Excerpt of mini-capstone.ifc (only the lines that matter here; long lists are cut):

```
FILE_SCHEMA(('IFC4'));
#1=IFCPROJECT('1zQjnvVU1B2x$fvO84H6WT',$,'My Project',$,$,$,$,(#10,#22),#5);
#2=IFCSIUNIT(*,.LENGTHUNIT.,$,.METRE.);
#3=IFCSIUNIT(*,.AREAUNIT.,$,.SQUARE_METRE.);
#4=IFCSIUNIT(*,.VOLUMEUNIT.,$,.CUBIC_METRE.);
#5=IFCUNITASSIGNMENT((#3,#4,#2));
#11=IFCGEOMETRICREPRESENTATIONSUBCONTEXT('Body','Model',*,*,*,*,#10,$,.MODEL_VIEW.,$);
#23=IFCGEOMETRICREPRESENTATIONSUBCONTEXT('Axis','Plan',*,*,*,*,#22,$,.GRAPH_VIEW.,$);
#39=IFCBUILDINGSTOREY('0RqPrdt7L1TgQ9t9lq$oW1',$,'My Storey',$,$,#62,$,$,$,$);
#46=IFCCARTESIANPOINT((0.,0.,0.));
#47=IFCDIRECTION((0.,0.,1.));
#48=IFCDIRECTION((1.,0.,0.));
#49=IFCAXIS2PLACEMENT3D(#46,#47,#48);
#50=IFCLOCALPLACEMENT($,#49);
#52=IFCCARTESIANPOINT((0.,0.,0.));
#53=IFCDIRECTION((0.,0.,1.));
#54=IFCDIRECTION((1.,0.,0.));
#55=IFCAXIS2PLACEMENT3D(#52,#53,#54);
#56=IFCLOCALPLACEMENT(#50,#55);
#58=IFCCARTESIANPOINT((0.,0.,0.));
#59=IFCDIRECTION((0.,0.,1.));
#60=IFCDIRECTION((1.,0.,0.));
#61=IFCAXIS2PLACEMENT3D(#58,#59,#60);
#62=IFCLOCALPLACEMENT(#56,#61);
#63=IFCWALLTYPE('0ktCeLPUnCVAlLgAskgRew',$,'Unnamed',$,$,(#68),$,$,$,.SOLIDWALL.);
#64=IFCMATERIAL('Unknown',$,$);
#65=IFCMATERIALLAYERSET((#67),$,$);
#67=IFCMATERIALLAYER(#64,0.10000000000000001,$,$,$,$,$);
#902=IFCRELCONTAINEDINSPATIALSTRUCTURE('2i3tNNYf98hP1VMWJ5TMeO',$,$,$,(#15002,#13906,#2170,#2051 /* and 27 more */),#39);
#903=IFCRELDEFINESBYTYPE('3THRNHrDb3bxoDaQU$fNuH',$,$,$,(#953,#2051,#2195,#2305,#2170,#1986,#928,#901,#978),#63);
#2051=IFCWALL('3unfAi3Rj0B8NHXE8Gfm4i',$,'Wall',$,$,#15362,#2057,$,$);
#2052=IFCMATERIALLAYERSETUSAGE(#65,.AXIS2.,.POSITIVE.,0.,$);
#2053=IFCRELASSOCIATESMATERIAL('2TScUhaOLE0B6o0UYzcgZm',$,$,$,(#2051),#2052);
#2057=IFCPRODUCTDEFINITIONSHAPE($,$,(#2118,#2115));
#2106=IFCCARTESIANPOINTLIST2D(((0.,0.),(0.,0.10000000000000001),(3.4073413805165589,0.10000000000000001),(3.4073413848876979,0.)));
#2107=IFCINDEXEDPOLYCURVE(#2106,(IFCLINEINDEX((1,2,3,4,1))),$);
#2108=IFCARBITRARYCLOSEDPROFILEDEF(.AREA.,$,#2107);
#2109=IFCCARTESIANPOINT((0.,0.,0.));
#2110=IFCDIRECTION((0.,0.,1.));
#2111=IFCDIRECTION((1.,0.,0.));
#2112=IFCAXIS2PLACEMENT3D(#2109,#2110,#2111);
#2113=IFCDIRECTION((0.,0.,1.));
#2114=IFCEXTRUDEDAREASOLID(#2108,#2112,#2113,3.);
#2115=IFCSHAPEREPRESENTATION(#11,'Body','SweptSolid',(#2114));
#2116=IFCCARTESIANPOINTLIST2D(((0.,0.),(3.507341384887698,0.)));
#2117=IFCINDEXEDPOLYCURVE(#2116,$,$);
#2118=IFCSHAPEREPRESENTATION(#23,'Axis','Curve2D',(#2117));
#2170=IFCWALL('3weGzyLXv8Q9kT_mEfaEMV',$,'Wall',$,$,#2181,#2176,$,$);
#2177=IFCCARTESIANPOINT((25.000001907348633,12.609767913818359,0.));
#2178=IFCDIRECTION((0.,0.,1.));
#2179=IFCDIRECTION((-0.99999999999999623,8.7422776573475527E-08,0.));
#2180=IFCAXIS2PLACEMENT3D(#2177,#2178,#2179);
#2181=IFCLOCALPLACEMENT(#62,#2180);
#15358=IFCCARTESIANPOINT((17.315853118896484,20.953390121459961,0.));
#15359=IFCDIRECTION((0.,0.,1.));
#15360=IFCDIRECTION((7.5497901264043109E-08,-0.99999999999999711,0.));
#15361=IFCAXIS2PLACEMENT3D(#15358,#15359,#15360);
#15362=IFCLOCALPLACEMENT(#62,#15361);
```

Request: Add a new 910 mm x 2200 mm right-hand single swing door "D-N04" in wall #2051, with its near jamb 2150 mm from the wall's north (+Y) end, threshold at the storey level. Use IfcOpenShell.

```python
import numpy as np
import ifcopenshell
import ifcopenshell.api.feature
import ifcopenshell.api.geometry
import ifcopenshell.api.root
import ifcopenshell.api.spatial
import ifcopenshell.geom
import ifcopenshell.util.element
import ifcopenshell.util.placement
import ifcopenshell.util.representation
import ifcopenshell.util.shape
import ifcopenshell.util.unit

model = ifcopenshell.open("mini-capstone.ifc")
unit_scale = ifcopenshell.util.unit.calculate_unit_scale(model)
settings = ifcopenshell.geom.settings()


def volume(element):
    """Net volume in cubic metres, openings subtracted."""
    shape = ifcopenshell.geom.create_shape(settings, element)
    return ifcopenshell.util.shape.get_volume(shape.geometry)


wall = model.by_id(2051)
storey = ifcopenshell.util.element.get_container(wall, ifc_class="IfcBuildingStorey")
context = ifcopenshell.util.representation.get_context(model, "Model", "Body", "MODEL_VIEW")
before = volume(wall)

width, height, from_end, sill = 0.91, 2.2, 2.15, 0.0  # metres

# The wall runs along its own X axis, and the end named is its -X end.
wall_shape = ifcopenshell.geom.create_shape(settings, wall)
x, y, z = ifcopenshell.util.shape.get_vertices(wall_shape.geometry).T
start = x.min() + from_end
face, thickness = float(y.min()), float(y.max() - y.min())
wall_matrix = ifcopenshell.util.placement.get_local_placement(wall.ObjectPlacement)
level = ifcopenshell.util.placement.get_local_placement(storey.ObjectPlacement)[2, 3]


def in_wall(x, y):
    """Placement at x, y metres in the wall's axes, at sill height."""
    matrix = wall_matrix.copy()
    matrix[:, 3] = wall_matrix @ np.array([x / unit_scale, y / unit_scale, 0.0, 1.0])
    matrix[2, 3] = level + sill / unit_scale
    return matrix


# Opening: a box that overshoots both wall faces by 50 mm.
opening = ifcopenshell.api.root.create_entity(model, ifc_class="IfcOpeningElement", predefined_type="OPENING")
box = ifcopenshell.api.geometry.add_wall_representation(
    model, context=context, length=width, height=height, thickness=thickness + 0.1
)
ifcopenshell.api.geometry.assign_representation(model, product=opening, representation=box)
ifcopenshell.api.geometry.edit_object_placement(model, product=opening, matrix=in_wall(start, face - 0.05), is_si=False)
ifcopenshell.api.feature.add_feature(model, feature=opening, element=wall)

door = ifcopenshell.api.root.create_entity(model, ifc_class="IfcDoor", name="D-N04", predefined_type="DOOR")
door.OverallWidth, door.OverallHeight = width / unit_scale, height / unit_scale
door.OperationType = "SINGLE_SWING_RIGHT"
body = ifcopenshell.api.geometry.add_door_representation(
    model,
    context=context,
    overall_width=door.OverallWidth,
    overall_height=door.OverallHeight,
    operation_type="SINGLE_SWING_RIGHT",
    lining_properties={"LiningDepth": thickness / unit_scale, "ThresholdDepth": thickness / unit_scale},
)
ifcopenshell.api.geometry.assign_representation(model, product=door, representation=body)
ifcopenshell.api.spatial.assign_container(model, products=[door], relating_structure=storey)
ifcopenshell.api.feature.add_filling(model, opening=opening, element=door)

# The lining spans the wall, so the door starts at the wall face.
ifcopenshell.api.geometry.edit_object_placement(model, product=door, matrix=in_wall(start, face), is_si=False)

after = volume(wall)

print(f"wall volume {before:.3f} -> {after:.3f} m3")

model.write("mini-capstone_rev.ifc")
```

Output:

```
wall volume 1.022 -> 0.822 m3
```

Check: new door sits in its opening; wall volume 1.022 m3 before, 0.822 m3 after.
